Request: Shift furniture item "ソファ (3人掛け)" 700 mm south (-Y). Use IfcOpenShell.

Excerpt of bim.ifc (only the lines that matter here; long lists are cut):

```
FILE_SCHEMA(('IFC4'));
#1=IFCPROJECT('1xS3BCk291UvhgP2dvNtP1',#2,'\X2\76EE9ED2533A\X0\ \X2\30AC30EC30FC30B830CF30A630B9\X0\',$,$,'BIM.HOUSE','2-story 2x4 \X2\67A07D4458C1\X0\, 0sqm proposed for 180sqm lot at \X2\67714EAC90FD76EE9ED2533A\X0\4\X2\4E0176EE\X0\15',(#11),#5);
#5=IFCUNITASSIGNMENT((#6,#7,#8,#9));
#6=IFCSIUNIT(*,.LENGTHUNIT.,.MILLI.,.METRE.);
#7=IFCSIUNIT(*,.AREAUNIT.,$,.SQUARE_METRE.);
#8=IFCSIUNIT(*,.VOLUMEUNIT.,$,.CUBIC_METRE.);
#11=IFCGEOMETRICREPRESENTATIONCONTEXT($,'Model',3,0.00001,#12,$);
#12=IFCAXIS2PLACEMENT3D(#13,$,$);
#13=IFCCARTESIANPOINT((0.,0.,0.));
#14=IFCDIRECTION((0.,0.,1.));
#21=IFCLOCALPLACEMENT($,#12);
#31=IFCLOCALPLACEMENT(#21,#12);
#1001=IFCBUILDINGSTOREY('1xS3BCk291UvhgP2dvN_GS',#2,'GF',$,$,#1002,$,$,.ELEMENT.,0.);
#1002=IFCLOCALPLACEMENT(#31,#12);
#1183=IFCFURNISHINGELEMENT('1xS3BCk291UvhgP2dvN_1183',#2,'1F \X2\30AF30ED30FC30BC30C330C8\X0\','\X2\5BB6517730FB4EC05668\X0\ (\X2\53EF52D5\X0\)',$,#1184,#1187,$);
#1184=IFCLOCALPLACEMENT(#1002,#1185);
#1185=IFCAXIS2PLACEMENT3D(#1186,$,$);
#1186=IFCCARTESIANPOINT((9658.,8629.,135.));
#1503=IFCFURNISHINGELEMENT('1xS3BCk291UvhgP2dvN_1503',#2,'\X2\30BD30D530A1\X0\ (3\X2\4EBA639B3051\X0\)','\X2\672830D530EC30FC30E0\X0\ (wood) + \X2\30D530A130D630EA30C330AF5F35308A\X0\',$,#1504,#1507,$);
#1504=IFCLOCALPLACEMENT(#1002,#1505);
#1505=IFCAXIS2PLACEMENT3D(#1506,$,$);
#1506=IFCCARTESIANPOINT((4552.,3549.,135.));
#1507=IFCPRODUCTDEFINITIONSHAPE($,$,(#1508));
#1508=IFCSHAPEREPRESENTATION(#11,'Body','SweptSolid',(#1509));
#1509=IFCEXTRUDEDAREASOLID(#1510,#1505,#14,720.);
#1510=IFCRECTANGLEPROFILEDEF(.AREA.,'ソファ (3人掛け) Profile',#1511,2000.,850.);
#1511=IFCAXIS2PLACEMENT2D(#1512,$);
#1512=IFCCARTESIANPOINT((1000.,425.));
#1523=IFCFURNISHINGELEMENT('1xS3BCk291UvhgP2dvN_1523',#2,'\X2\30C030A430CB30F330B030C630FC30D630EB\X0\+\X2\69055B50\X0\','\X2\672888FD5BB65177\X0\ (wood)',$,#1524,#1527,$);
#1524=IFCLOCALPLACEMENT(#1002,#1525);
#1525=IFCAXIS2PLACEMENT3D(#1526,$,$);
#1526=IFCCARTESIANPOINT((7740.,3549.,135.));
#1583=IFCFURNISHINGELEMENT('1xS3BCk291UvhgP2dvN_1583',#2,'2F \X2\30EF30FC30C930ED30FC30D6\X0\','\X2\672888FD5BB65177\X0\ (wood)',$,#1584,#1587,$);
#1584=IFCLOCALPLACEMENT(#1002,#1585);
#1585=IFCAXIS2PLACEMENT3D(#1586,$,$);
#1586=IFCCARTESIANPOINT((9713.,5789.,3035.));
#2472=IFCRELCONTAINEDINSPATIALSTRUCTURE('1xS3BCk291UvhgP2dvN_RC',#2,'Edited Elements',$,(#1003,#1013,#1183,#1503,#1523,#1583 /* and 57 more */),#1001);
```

```python
import ifcopenshell
import ifcopenshell.api.geometry
import ifcopenshell.util.placement

model = ifcopenshell.open("bim.ifc")

item = model.by_guid("1xS3BCk291UvhgP2dvN_1503")
matrix = ifcopenshell.util.placement.get_local_placement(item.ObjectPlacement)
matrix[1, 3] -= 700.0
ifcopenshell.api.geometry.edit_object_placement(model, product=item, matrix=matrix, is_si=False)

print(ifcopenshell.util.placement.get_local_placement(item.ObjectPlacement).round(3) + 0.0)

model.write("bim_updated.ifc")
```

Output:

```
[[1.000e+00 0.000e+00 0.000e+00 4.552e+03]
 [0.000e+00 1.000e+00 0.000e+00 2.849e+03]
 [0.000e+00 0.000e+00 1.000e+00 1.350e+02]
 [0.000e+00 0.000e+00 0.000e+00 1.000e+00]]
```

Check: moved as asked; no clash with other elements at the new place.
